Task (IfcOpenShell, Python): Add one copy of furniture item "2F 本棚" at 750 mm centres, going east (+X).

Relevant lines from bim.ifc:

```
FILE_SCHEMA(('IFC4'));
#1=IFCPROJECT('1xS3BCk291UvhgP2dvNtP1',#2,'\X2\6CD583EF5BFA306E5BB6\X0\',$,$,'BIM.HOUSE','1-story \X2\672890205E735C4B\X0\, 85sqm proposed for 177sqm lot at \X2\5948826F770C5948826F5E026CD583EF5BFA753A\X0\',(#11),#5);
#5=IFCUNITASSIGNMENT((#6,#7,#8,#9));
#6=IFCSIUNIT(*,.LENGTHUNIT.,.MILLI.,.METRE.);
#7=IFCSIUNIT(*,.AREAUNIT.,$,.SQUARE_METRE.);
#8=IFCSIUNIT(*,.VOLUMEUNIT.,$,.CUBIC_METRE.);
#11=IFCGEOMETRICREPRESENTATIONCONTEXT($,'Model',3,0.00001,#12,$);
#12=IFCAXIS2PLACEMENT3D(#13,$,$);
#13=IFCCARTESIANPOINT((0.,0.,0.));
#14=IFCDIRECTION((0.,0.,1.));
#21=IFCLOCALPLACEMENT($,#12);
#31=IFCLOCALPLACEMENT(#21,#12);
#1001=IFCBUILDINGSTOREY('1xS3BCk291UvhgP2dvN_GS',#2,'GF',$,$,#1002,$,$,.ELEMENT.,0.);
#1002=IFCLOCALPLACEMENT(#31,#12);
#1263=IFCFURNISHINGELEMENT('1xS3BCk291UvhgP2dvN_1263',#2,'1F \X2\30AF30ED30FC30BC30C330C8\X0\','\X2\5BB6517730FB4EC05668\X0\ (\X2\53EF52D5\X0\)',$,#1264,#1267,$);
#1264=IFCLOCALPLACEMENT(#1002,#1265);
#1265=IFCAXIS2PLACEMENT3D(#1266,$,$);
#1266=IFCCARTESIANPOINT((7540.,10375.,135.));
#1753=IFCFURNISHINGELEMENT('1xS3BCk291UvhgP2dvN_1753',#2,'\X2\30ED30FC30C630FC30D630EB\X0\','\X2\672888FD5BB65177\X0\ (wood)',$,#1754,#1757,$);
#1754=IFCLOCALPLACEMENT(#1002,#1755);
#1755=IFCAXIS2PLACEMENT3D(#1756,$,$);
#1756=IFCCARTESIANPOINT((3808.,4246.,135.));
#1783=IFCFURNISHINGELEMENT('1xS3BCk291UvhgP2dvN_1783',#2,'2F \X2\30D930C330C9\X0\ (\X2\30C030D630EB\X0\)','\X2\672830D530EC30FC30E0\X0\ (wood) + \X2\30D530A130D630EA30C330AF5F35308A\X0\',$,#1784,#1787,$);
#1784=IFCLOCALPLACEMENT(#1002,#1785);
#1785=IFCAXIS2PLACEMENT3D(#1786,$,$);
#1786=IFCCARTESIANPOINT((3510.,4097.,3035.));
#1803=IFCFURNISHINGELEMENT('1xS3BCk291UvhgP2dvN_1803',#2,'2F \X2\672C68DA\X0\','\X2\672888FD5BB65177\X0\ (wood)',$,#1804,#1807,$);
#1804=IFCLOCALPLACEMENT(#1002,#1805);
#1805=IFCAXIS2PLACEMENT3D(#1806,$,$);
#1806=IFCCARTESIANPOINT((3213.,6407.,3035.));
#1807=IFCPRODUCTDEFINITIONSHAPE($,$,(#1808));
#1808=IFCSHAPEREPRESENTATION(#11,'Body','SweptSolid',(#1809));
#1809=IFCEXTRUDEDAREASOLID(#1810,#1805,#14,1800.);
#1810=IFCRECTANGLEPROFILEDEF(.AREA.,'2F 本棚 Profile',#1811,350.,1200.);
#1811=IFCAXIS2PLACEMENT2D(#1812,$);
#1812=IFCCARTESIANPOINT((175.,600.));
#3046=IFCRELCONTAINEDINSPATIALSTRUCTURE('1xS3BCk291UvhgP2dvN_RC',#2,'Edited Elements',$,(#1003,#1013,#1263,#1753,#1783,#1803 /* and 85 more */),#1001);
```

```python
import numpy as np
import ifcopenshell
import ifcopenshell.api.geometry
import ifcopenshell.api.root
import ifcopenshell.util.element
import ifcopenshell.util.placement

model = ifcopenshell.open("bim.ifc")


def reuse_history(source, copy):
    """copy_class also copies each property set's owner history, people and application; keep the originals."""
    for rel in copy.IsDefinedBy:
        if rel.is_a("IfcRelDefinesByProperties") and (history := rel.RelatingPropertyDefinition.OwnerHistory):
            rel.RelatingPropertyDefinition.OwnerHistory = source.OwnerHistory
            ifcopenshell.util.element.remove_deep2(model, history)


source = model.by_id(1803)
base = ifcopenshell.util.placement.get_local_placement(source.ObjectPlacement)
step = np.array([1.0, 0.0, 0.0]) * 750.0

for i in range(1, 2):
    copy = ifcopenshell.api.root.copy_class(model, product=source)
    copy.Representation = ifcopenshell.util.element.copy_deep(
        model, source.Representation, exclude=["IfcGeometricRepresentationContext", "IfcRepresentationMap"]
    )
    reuse_history(source, copy)
    matrix = base.copy()
    matrix[:3, 3] += i * step
    print("added at", matrix[:3, 3].round(3) + 0.0)
    ifcopenshell.api.geometry.edit_object_placement(model, product=copy, matrix=matrix, is_si=False)

model.write("bim_v2.ifc")
```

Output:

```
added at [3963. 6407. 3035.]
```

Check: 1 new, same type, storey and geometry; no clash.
